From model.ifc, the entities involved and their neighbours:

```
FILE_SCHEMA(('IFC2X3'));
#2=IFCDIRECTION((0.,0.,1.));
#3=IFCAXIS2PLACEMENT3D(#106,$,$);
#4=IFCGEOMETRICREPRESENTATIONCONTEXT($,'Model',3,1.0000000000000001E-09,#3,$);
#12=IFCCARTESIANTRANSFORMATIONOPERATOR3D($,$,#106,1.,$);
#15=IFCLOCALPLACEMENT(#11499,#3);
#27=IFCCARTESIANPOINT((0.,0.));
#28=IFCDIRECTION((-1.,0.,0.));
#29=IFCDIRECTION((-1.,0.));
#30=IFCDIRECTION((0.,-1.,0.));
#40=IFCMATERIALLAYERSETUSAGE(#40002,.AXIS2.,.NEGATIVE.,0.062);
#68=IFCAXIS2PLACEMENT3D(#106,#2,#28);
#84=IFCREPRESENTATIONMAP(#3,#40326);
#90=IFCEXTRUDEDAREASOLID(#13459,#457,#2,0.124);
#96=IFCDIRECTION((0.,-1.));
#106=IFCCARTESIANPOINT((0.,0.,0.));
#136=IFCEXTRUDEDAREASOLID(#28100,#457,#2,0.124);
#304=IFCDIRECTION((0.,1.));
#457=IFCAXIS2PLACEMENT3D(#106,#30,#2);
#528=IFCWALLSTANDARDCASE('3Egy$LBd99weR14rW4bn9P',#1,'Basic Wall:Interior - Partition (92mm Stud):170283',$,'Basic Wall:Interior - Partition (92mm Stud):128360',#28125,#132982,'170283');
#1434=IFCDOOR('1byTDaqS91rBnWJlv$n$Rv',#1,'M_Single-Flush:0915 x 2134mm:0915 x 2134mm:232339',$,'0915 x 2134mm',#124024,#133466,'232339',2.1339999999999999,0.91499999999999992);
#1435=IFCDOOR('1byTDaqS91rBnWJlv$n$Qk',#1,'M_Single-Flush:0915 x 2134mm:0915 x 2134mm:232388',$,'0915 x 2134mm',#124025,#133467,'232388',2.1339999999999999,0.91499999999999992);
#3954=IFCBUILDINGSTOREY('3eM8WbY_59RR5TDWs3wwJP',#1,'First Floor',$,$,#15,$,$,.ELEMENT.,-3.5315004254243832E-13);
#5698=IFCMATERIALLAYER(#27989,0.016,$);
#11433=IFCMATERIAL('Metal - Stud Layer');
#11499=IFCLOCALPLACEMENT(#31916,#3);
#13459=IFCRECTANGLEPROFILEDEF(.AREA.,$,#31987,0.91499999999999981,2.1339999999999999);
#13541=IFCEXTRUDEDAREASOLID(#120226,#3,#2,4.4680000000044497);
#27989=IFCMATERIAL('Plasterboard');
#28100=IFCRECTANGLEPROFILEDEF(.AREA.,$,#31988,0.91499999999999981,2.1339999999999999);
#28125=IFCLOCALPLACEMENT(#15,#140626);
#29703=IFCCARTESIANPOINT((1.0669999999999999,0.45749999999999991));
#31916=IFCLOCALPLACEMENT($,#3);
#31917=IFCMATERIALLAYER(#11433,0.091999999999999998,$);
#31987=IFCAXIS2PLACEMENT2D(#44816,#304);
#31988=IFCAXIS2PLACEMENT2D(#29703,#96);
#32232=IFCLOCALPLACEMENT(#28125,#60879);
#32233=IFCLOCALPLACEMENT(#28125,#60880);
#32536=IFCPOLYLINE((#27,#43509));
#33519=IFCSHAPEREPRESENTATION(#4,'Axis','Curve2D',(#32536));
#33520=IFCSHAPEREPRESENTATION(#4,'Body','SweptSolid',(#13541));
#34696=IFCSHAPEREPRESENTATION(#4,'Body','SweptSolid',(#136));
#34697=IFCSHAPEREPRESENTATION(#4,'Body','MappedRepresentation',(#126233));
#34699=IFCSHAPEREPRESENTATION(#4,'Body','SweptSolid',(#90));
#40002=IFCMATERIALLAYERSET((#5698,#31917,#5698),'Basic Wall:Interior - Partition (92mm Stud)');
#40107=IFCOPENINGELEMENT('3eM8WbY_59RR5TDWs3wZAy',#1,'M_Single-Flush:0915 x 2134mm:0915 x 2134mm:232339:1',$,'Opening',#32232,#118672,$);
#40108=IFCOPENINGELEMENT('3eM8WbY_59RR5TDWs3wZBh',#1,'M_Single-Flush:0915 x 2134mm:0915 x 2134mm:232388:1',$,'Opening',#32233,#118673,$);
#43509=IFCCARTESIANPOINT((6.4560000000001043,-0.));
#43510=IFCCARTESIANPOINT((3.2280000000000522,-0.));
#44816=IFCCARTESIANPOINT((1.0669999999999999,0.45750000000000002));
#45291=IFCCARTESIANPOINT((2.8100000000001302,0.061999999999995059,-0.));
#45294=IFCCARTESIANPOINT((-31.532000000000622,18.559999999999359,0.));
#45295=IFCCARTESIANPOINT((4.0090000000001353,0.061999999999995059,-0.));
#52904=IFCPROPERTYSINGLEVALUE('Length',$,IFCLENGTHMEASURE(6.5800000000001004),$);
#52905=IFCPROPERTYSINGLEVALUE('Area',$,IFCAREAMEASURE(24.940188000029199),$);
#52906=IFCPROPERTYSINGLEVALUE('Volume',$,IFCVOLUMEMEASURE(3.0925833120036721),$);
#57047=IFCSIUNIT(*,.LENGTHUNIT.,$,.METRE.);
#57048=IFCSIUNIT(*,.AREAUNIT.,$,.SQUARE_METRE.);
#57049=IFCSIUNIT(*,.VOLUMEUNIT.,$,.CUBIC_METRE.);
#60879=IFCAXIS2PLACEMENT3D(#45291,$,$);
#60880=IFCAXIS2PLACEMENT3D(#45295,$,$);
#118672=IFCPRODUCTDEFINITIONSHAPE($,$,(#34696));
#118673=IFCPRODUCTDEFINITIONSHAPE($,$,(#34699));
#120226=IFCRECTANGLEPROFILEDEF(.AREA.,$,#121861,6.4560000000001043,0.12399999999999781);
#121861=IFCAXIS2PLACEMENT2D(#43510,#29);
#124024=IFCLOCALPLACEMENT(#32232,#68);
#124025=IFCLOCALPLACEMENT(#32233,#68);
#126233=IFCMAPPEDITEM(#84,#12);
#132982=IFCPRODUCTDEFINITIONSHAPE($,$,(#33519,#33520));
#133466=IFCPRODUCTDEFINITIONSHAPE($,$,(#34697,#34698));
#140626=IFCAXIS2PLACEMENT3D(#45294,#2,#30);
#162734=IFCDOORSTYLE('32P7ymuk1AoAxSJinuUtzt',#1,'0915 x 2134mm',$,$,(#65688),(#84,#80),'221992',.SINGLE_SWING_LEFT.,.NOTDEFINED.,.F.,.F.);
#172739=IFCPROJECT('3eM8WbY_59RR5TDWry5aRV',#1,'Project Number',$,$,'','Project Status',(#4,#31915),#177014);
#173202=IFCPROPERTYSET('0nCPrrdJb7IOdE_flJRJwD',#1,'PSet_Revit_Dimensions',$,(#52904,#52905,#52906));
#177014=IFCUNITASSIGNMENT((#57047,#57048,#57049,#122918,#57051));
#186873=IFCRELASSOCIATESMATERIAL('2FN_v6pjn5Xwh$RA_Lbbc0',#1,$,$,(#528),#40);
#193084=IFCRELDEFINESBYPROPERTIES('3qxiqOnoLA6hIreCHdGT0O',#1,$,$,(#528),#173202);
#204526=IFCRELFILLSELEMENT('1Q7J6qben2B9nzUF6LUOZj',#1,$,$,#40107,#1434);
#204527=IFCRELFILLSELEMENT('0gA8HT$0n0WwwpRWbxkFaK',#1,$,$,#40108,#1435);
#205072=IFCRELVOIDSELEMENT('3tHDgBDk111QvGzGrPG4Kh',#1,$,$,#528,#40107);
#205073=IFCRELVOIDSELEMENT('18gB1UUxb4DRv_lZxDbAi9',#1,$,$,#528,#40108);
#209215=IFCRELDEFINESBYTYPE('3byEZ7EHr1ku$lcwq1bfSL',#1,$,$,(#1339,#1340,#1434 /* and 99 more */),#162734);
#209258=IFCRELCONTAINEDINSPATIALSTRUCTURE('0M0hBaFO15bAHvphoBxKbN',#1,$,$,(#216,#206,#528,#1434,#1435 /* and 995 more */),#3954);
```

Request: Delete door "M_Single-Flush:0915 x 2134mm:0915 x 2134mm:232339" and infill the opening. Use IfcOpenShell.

```python
import ifcopenshell
import ifcopenshell.api.feature
import ifcopenshell.api.pset
import ifcopenshell.api.root
import ifcopenshell.geom
import ifcopenshell.util.element
import ifcopenshell.util.shape
import ifcopenshell.util.unit

model = ifcopenshell.open("model.ifc")
area_scale = ifcopenshell.util.unit.calculate_unit_scale(model, "AREAUNIT")
volume_scale = ifcopenshell.util.unit.calculate_unit_scale(model, "VOLUMEUNIT")
settings = ifcopenshell.geom.settings()


def volume(element):
    """Net volume in cubic metres, openings subtracted."""
    shape = ifcopenshell.geom.create_shape(settings, element)
    return ifcopenshell.util.shape.get_volume(shape.geometry)


door = model.by_id(1434)
opening = door.FillsVoids[0].RelatingOpeningElement
wall = opening.VoidsElements[0].RelatingBuildingElement
before = volume(wall)

ifcopenshell.api.root.remove_product(model, product=door)
ifcopenshell.api.feature.remove_feature(model, feature=opening)

after = volume(wall)
thickness = 0.124  # wall thickness in metres

# Update the wall's stored quantities.
pset = model.by_id(ifcopenshell.util.element.get_pset(wall, "PSet_Revit_Dimensions", should_inherit=False)["id"])
ifcopenshell.api.pset.edit_pset(model, pset=pset, properties={
    "Area": model.create_entity("IfcAreaMeasure", after / thickness / area_scale),
    "Volume": model.create_entity("IfcVolumeMeasure", after / volume_scale),
})

print(f"wall volume {before:.3f} -> {after:.3f} m3")

model.write("model_v2.ifc")
```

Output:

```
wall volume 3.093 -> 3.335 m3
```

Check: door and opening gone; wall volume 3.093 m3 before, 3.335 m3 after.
